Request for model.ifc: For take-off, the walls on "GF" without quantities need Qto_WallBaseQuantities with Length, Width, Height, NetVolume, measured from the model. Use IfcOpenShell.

First a look at what the model holds.

```python
import ifcopenshell
import ifcopenshell.util.element
import ifcopenshell.util.unit

model = ifcopenshell.open("model.ifc")
print(model.schema)
for unit_type in ("LENGTHUNIT", "AREAUNIT", "VOLUMEUNIT"):
    print(unit_type, ifcopenshell.util.unit.calculate_unit_scale(model, unit_type))
storey = next(s for s in model.by_type("IfcBuildingStorey") if s.Name == "GF")
walls = [e for e in ifcopenshell.util.element.get_decomposition(storey) if e.is_a("IfcWall")]
for e in sorted(walls, key=lambda e: e.id()):
    print(e.id(), e.is_a(), e.Name, list(ifcopenshell.util.element.get_psets(e, qtos_only=True)), sep=" | ")
```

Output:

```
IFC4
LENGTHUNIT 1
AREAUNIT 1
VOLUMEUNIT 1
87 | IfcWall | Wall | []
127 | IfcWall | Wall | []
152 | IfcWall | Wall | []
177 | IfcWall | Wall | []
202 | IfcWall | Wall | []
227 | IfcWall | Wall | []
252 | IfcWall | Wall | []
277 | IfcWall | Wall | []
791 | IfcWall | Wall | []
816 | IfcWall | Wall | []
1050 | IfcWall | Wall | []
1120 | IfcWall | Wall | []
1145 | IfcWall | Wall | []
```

```python
import ifcopenshell
import ifcopenshell.api.pset
import ifcopenshell.geom
import ifcopenshell.util.element
import ifcopenshell.util.shape
import ifcopenshell.util.unit

model = ifcopenshell.open("model.ifc")
unit_scale = ifcopenshell.util.unit.calculate_unit_scale(model)
volume_scale = ifcopenshell.util.unit.calculate_unit_scale(model, "VOLUMEUNIT")
settings = ifcopenshell.geom.settings()

storey = next(s for s in model.by_type("IfcBuildingStorey") if s.Name == "GF")
walls = [e for e in ifcopenshell.util.element.get_decomposition(storey) if e.is_a("IfcWall")]

for e in sorted(walls, key=lambda e: e.id()):
    if ifcopenshell.util.element.get_psets(e, qtos_only=True, should_inherit=False):
        continue
    # Geometry comes back in metres, in the element's own axes.
    shape = ifcopenshell.geom.create_shape(settings, e)
    values = {
        "Length": ifcopenshell.util.shape.get_x(shape.geometry) / unit_scale,
        "Width": ifcopenshell.util.shape.get_y(shape.geometry) / unit_scale,
        "Height": ifcopenshell.util.shape.get_z(shape.geometry) / unit_scale,
        "NetVolume": ifcopenshell.util.shape.get_volume(shape.geometry) / volume_scale,
    }
    qto = ifcopenshell.api.pset.add_qto(model, product=e, name="Qto_WallBaseQuantities")
    ifcopenshell.api.pset.edit_qto(model, qto=qto, properties=values)
    print(e.id(), {k: round(v, 3) for k, v in values.items()})

model.write("model_v2.ifc")
```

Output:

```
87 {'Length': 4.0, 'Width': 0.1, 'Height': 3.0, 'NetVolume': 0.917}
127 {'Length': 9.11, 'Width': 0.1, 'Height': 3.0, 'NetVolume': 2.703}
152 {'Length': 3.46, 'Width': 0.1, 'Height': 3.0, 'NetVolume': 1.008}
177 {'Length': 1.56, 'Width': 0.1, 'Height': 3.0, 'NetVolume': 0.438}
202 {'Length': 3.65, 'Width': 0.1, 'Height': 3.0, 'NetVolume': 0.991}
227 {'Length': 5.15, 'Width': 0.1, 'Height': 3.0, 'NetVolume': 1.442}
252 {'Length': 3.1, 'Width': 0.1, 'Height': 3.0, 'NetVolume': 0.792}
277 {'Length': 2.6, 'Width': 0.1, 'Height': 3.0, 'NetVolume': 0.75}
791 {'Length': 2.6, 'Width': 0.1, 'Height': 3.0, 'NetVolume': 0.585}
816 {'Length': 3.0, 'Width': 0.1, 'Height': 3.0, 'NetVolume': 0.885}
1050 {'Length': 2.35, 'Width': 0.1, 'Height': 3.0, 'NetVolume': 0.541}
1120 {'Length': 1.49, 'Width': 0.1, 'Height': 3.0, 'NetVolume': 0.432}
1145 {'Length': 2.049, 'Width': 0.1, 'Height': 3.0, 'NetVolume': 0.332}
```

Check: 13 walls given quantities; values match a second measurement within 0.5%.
